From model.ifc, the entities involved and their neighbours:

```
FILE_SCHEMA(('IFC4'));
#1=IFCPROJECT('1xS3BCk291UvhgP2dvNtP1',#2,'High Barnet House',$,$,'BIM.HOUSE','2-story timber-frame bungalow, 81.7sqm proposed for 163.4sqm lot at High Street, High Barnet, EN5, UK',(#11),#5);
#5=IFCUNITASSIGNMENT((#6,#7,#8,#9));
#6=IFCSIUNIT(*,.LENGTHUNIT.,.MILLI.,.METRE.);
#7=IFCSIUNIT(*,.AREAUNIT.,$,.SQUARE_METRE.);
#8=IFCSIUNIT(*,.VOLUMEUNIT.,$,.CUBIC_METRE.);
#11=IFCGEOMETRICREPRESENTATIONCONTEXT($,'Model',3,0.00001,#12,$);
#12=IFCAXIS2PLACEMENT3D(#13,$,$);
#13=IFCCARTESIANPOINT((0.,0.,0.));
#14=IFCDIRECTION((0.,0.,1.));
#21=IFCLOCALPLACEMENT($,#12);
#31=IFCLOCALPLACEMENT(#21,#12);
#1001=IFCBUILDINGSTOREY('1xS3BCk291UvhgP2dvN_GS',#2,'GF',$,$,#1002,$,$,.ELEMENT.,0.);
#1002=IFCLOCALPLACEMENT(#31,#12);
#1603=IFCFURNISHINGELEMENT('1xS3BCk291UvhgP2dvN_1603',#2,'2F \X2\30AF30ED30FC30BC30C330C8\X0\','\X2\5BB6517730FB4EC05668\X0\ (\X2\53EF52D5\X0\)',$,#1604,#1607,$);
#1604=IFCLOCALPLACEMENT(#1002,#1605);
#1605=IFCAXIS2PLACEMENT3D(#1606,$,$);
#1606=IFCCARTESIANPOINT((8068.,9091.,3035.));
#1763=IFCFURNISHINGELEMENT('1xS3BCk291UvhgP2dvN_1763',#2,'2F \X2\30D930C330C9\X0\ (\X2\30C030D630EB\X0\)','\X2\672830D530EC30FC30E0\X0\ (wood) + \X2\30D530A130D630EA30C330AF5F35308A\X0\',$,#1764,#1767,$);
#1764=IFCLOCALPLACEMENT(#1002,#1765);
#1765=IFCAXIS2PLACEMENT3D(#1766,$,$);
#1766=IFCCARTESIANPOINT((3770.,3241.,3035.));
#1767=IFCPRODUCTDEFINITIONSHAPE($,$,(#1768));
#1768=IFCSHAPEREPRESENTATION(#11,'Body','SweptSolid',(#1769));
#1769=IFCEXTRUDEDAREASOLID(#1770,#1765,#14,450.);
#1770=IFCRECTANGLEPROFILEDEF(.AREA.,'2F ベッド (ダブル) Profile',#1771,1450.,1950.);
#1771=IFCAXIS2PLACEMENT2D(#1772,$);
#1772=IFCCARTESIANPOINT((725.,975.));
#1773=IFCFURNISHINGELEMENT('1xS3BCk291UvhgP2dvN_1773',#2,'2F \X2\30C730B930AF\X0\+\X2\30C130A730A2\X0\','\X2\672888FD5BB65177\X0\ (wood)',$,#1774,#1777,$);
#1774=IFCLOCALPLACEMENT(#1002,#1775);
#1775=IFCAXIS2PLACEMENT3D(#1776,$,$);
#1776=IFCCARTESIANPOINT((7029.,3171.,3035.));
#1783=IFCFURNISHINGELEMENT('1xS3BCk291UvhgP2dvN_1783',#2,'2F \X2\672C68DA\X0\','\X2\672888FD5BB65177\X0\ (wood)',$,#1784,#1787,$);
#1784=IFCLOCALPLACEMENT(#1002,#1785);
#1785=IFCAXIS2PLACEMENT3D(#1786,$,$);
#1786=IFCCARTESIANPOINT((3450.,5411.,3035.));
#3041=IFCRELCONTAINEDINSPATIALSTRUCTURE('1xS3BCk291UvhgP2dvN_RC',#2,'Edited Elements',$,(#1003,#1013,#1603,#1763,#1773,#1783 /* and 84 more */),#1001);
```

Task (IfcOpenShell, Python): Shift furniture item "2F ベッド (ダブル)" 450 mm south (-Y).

```python
import ifcopenshell
import ifcopenshell.api.geometry
import ifcopenshell.util.placement

model = ifcopenshell.open("model.ifc")

item = model.by_id(1763)
matrix = ifcopenshell.util.placement.get_local_placement(item.ObjectPlacement)
matrix[1, 3] -= 450.0
ifcopenshell.api.geometry.edit_object_placement(model, product=item, matrix=matrix, is_si=False)

print(ifcopenshell.util.placement.get_local_placement(item.ObjectPlacement).round(3) + 0.0)

model.write("model-out.ifc")
```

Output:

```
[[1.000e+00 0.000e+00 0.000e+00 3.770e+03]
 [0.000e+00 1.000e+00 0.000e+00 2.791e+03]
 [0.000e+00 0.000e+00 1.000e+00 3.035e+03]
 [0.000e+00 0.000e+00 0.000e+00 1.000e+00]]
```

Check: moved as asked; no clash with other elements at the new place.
